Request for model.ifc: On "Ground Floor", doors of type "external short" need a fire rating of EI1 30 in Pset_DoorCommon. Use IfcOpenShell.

First a look at what the model holds.

```python
import ifcopenshell
import ifcopenshell.util.element

model = ifcopenshell.open("model.ifc")
print(model.schema)
storey = next(s for s in model.by_type("IfcBuildingStorey") if s.Name == "Ground Floor")
doors = [e for e in ifcopenshell.util.element.get_decomposition(storey) if e.is_a("IfcDoor")]
seen = {}
for e in doors:
    element_type = ifcopenshell.util.element.get_type(e)
    key = (element_type.Name if element_type != e and element_type else None, ifcopenshell.util.element.get_pset(e, "Pset_DoorCommon", "FireRating"))
    seen[key] = seen.get(key, 0) + 1
for (name, value), count in sorted(seen.items(), key=str):
    print(count, "x", name, "|", value)
```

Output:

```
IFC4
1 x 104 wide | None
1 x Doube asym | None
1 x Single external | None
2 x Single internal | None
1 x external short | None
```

```python
import ifcopenshell
import ifcopenshell.api.pset
import ifcopenshell.util.element

model = ifcopenshell.open("model.ifc")

storey = next(s for s in model.by_type("IfcBuildingStorey") if s.Name == "Ground Floor")
doors = [e for e in ifcopenshell.util.element.get_decomposition(storey) if e.is_a("IfcDoor")]

count = 0
for e in doors:
    element_type = ifcopenshell.util.element.get_type(e)
    if element_type in (None, e) or element_type.Name != "external short":
        continue
    # add_pset returns the element's existing set when there is one.
    pset = ifcopenshell.api.pset.add_pset(model, product=e, name="Pset_DoorCommon")
    ifcopenshell.api.pset.edit_pset(model, pset=pset, properties={"FireRating": "EI1 30"})
    count += 1

print(count, "doors updated")

model.write("model_edited.ifc")
```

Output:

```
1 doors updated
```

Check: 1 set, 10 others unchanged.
